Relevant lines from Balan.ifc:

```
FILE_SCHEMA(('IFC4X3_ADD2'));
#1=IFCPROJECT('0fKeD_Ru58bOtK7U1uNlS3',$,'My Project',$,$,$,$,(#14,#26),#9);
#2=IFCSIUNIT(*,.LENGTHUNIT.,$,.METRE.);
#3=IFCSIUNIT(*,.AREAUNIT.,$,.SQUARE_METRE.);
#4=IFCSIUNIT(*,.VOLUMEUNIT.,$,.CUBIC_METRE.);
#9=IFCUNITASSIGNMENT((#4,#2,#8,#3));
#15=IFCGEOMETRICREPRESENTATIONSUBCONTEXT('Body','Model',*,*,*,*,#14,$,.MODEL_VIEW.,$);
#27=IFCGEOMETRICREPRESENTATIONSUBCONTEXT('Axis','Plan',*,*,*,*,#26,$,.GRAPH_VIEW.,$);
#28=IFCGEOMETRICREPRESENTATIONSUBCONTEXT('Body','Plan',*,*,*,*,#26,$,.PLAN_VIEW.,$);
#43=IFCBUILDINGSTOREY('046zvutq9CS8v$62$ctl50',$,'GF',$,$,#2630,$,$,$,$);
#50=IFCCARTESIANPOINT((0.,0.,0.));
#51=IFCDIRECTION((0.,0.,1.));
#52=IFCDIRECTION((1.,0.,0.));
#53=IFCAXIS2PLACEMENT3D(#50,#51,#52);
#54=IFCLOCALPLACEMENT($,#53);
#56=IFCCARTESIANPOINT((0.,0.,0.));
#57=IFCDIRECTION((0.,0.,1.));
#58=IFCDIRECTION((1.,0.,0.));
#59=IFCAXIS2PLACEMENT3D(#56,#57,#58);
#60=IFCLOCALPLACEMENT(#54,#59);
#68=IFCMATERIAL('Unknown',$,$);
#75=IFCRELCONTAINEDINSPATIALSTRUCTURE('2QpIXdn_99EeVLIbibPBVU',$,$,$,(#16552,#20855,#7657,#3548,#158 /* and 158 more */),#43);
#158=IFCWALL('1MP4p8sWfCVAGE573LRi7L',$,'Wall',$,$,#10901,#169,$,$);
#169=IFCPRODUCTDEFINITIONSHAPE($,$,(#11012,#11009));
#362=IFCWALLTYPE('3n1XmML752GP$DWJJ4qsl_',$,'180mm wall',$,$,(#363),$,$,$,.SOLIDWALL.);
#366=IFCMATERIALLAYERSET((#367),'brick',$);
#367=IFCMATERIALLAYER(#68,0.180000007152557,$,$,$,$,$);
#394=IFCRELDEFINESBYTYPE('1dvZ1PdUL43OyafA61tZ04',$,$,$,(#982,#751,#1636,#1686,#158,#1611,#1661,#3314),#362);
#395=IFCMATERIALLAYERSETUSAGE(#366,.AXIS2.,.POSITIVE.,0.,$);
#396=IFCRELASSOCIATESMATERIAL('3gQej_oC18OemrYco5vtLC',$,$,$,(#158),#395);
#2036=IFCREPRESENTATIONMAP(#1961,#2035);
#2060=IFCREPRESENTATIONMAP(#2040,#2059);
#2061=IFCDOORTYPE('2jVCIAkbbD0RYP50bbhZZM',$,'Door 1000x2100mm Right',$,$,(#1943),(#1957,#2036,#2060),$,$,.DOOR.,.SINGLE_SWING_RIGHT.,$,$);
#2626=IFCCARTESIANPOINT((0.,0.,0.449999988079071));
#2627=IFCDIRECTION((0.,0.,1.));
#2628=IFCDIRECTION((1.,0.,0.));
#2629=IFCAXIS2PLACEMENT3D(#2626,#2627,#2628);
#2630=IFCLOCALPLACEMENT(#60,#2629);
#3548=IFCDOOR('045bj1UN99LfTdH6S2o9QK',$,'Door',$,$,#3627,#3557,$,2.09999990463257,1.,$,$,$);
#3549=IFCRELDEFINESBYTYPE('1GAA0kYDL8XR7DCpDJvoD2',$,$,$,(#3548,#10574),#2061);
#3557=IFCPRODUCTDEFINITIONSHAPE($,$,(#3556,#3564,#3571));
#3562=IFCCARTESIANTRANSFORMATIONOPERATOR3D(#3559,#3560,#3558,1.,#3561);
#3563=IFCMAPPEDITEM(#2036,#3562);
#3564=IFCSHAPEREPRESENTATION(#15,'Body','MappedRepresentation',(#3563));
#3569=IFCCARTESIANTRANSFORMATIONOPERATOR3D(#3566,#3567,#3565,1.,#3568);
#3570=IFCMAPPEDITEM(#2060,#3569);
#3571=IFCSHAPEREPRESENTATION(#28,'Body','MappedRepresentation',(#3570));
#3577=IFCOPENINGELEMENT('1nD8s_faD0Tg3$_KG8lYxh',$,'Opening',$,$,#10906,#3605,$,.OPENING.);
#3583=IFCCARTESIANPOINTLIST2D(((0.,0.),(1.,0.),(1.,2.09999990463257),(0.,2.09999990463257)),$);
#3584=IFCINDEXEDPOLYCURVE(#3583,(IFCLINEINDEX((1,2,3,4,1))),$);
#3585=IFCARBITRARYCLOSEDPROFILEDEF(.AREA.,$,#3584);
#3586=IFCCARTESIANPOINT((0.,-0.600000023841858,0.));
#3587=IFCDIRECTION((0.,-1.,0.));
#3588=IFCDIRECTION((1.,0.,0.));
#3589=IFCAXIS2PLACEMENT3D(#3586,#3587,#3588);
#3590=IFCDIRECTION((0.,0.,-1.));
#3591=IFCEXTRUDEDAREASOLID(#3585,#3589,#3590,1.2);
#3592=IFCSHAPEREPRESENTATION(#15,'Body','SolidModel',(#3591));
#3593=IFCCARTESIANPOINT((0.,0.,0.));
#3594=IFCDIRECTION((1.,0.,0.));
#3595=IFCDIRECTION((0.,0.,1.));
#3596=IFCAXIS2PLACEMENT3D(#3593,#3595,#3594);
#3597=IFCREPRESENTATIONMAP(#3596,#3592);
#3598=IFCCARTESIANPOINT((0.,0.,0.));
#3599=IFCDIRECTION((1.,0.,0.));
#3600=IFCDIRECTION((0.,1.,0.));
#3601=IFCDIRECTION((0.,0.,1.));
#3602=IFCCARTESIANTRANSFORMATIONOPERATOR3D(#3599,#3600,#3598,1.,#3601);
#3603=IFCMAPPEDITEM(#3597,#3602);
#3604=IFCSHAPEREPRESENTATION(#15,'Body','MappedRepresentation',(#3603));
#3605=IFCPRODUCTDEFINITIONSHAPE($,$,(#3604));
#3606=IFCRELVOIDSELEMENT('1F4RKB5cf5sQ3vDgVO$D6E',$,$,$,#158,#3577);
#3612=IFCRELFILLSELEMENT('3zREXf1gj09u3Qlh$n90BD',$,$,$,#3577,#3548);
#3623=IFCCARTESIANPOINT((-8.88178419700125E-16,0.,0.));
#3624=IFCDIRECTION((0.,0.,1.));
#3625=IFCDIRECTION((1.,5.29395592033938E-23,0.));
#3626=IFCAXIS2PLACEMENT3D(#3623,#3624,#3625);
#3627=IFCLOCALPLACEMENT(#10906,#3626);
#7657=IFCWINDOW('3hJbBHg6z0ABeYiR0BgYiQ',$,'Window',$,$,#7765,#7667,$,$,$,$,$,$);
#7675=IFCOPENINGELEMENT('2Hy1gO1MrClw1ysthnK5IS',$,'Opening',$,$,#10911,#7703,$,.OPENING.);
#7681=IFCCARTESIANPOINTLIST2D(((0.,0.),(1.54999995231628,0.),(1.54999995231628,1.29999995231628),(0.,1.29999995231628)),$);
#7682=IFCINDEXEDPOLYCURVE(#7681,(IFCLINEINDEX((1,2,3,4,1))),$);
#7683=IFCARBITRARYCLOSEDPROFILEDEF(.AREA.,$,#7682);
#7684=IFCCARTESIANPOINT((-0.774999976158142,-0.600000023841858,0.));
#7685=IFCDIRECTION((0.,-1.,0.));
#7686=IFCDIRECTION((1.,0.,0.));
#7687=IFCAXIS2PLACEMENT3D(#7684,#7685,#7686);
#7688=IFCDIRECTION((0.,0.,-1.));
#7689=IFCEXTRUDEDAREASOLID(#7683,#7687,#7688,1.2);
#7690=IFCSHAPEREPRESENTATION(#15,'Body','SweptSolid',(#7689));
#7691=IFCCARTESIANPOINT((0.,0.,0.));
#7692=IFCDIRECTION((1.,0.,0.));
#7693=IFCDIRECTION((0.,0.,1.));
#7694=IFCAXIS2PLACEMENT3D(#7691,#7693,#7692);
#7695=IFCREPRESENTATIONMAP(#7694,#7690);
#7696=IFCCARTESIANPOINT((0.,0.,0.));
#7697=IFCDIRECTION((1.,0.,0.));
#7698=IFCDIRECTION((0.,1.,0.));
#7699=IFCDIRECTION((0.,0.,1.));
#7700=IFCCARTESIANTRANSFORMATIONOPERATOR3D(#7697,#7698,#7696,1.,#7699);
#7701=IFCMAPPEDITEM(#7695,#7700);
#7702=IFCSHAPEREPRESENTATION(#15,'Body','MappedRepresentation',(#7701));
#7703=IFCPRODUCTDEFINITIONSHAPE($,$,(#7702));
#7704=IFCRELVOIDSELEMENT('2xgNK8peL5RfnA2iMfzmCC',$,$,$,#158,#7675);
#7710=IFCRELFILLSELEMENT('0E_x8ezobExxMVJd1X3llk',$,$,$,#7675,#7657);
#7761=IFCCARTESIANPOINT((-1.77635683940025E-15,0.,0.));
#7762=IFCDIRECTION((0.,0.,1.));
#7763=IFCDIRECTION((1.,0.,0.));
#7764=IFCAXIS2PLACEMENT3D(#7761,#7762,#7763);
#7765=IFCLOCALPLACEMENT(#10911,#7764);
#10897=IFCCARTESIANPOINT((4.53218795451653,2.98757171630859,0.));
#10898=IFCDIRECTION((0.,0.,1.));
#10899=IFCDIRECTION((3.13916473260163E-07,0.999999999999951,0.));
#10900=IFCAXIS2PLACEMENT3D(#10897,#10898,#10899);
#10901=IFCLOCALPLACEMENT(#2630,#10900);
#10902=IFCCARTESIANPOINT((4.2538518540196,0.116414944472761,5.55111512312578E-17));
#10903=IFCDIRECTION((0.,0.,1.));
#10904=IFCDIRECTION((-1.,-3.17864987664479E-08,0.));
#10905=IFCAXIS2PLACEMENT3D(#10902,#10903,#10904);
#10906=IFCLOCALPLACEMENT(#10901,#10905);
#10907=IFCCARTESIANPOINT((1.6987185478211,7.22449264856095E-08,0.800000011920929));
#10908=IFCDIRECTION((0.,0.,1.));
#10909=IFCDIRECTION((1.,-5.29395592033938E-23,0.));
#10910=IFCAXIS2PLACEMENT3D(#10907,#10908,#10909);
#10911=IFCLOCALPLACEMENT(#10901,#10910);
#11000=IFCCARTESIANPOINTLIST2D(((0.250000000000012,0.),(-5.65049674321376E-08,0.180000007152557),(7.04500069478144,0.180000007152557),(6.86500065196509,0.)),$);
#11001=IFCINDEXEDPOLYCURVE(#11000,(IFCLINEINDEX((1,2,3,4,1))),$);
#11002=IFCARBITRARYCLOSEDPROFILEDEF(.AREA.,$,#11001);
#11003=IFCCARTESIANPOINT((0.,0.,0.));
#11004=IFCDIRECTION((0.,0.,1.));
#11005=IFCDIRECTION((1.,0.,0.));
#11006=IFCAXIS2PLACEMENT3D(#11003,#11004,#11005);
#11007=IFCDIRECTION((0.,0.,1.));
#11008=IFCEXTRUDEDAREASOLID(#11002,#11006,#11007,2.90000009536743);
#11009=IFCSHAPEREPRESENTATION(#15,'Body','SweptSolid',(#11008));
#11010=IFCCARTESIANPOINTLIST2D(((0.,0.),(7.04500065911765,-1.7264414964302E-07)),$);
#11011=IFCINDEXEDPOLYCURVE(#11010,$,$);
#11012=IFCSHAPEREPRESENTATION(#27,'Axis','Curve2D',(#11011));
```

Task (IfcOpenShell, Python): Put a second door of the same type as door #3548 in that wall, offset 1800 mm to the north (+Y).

```python
import ifcopenshell
import ifcopenshell.api.feature
import ifcopenshell.api.geometry
import ifcopenshell.api.root
import ifcopenshell.geom
import ifcopenshell.util.element
import ifcopenshell.util.placement
import ifcopenshell.util.shape
import ifcopenshell.util.unit

model = ifcopenshell.open("Balan.ifc")
unit_scale = ifcopenshell.util.unit.calculate_unit_scale(model)
settings = ifcopenshell.geom.settings()


def volume(element):
    """Net volume in cubic metres, openings subtracted."""
    shape = ifcopenshell.geom.create_shape(settings, element)
    return ifcopenshell.util.shape.get_volume(shape.geometry)


door = model.by_guid("045bj1UN99LfTdH6S2o9QK")
opening = door.FillsVoids[0].RelatingOpeningElement
wall = opening.VoidsElements[0].RelatingBuildingElement
before = volume(wall)
shift = ifcopenshell.util.placement.get_local_placement(wall.ObjectPlacement)[:3, 0] * 1.8 / unit_scale

# copy_class copies the void relationship, type, container and properties, but no geometry.
new_opening = ifcopenshell.api.root.copy_class(model, product=opening)
new_opening.Representation = ifcopenshell.util.element.copy_deep(
    model, opening.Representation, exclude=["IfcGeometricRepresentationContext", "IfcRepresentationMap"]
)
new_door = ifcopenshell.api.root.copy_class(model, product=door)
new_door.Representation = ifcopenshell.util.element.copy_deep(
    model, door.Representation, exclude=["IfcGeometricRepresentationContext", "IfcRepresentationMap"]
)
ifcopenshell.api.feature.add_filling(model, opening=new_opening, element=new_door)

for old, new in ((opening, new_opening), (door, new_door)):
    matrix = ifcopenshell.util.placement.get_local_placement(old.ObjectPlacement)
    matrix[:3, 3] += shift
    ifcopenshell.api.geometry.edit_object_placement(model, product=new, matrix=matrix, is_si=False)

after = volume(wall)

print(f"wall volume {before:.3f} -> {after:.3f} m3")

model.write("Balan_v2.ifc")
```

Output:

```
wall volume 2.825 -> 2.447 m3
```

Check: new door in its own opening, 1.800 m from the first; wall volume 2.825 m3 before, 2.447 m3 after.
